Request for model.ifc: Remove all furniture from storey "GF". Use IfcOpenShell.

First a look at what the model holds.

```python
import ifcopenshell
import ifcopenshell.util.element

model = ifcopenshell.open("model.ifc")
print(model.schema)
storey = next(s for s in model.by_type("IfcBuildingStorey") if s.Name == "GF")
furniture = [e for e in ifcopenshell.util.element.get_decomposition(storey) if e.is_a("IfcFurnishingElement")]
seen = {}
for e in furniture:
    element_type = ifcopenshell.util.element.get_type(e)
    name = element_type.Name if element_type not in (None, e) else None
    seen[name] = seen.get(name, 0) + 1
for name, count in sorted(seen.items(), key=str):
    print(count, "x", name)
```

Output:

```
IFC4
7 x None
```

```python
import ifcopenshell
import ifcopenshell.api.root
import ifcopenshell.util.element

model = ifcopenshell.open("model.ifc")

storey = next(s for s in model.by_type("IfcBuildingStorey") if s.Name == "GF")
furniture = [e for e in ifcopenshell.util.element.get_decomposition(storey) if e.is_a("IfcFurnishingElement")]

for e in furniture:
    ifcopenshell.api.root.remove_product(model, product=e)
print(len(furniture), "removed")

model.write("model_updated.ifc")
```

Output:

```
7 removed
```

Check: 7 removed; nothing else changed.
